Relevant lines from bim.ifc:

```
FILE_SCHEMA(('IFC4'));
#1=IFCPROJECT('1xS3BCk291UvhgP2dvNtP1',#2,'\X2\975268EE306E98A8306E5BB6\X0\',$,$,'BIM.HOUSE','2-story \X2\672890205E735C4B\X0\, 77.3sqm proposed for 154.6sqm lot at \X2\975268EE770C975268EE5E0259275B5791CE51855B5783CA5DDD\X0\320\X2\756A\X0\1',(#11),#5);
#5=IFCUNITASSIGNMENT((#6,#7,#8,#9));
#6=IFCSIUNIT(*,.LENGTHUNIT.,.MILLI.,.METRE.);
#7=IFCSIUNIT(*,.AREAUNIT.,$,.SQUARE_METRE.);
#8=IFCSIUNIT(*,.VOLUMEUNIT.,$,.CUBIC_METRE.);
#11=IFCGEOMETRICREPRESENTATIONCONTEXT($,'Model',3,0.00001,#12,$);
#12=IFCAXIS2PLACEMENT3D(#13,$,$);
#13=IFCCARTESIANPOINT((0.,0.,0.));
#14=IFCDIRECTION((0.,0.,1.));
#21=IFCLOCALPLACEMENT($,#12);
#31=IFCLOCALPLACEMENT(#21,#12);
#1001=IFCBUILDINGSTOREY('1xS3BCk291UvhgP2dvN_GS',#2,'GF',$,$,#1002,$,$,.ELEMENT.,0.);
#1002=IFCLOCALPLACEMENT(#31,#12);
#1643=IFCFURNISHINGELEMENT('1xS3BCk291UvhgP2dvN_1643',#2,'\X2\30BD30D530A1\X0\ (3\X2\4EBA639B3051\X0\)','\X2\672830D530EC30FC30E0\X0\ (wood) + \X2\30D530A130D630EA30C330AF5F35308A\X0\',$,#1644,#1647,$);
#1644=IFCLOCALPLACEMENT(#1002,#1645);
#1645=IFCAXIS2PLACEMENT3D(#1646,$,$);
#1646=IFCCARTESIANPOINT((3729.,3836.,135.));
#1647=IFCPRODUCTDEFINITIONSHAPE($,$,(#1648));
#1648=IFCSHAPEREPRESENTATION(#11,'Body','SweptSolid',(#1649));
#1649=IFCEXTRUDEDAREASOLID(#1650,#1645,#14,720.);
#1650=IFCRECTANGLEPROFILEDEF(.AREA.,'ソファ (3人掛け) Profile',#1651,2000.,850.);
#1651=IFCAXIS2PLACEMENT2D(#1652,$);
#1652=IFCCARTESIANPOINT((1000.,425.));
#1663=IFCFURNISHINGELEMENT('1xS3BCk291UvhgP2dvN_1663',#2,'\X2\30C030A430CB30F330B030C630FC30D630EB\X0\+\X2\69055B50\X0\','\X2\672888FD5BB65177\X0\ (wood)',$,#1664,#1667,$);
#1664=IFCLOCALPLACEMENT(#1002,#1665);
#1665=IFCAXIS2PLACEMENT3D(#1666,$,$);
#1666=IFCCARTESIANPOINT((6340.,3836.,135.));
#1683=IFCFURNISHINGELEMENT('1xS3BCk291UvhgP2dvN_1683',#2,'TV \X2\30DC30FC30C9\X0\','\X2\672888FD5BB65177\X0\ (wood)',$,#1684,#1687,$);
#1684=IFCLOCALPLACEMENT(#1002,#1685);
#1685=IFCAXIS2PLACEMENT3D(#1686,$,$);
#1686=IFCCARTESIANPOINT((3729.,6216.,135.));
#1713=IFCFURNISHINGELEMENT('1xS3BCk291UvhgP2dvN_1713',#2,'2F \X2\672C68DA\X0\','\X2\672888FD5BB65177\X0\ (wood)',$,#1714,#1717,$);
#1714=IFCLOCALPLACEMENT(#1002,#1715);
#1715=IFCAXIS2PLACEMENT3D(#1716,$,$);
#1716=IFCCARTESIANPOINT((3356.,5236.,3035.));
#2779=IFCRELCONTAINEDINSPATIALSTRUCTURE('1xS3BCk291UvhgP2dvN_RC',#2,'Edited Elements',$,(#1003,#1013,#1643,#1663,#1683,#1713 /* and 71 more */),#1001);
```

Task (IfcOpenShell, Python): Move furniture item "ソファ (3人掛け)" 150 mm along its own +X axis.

```python
import ifcopenshell
import ifcopenshell.api.geometry
import ifcopenshell.util.placement

model = ifcopenshell.open("bim.ifc")

item = model.by_guid("1xS3BCk291UvhgP2dvN_1643")
matrix = ifcopenshell.util.placement.get_local_placement(item.ObjectPlacement)
matrix[:3, 3] += matrix[:3, 0] * 150.0
ifcopenshell.api.geometry.edit_object_placement(model, product=item, matrix=matrix, is_si=False)

print(ifcopenshell.util.placement.get_local_placement(item.ObjectPlacement).round(3) + 0.0)

model.write("bim_rev.ifc")
```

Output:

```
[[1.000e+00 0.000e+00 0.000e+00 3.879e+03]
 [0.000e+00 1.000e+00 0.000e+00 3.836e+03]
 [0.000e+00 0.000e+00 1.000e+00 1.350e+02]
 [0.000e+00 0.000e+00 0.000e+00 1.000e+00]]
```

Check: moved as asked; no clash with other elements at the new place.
